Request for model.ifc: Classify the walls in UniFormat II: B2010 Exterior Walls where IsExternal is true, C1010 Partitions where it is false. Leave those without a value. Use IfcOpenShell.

First a look at what the model holds.

```python
import ifcopenshell
import ifcopenshell.util.element

model = ifcopenshell.open("model.ifc")
print(model.schema)
print("classifications:", [c.Name for c in model.by_type("IfcClassification")])
values = [ifcopenshell.util.element.get_pset(e, "Pset_WallCommon", "IsExternal") for e in model.by_type("IfcWall")]
for value in (True, False, None):
    print("IsExternal", value, values.count(value))
```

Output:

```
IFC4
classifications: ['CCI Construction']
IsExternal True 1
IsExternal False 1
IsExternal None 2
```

```python
import ifcopenshell
import ifcopenshell.api.classification
import ifcopenshell.util.element

model = ifcopenshell.open("model.ifc")

system = ifcopenshell.api.classification.add_classification(model, classification="UniFormat II")

walls = model.by_type("IfcWall")
external = {e: ifcopenshell.util.element.get_pset(e, "Pset_WallCommon", "IsExternal") for e in walls}
for flag, code, name in ((True, "B2010", "Exterior Walls"), (False, "C1010", "Partitions")):
    products = [e for e in walls if external[e] is flag]
    ifcopenshell.api.classification.add_reference(
        model, products=products, classification=system, identification=code, name=name
    )
    print(code, len(products))

model.write("model_rev.ifc")
```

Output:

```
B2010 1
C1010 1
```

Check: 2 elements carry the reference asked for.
